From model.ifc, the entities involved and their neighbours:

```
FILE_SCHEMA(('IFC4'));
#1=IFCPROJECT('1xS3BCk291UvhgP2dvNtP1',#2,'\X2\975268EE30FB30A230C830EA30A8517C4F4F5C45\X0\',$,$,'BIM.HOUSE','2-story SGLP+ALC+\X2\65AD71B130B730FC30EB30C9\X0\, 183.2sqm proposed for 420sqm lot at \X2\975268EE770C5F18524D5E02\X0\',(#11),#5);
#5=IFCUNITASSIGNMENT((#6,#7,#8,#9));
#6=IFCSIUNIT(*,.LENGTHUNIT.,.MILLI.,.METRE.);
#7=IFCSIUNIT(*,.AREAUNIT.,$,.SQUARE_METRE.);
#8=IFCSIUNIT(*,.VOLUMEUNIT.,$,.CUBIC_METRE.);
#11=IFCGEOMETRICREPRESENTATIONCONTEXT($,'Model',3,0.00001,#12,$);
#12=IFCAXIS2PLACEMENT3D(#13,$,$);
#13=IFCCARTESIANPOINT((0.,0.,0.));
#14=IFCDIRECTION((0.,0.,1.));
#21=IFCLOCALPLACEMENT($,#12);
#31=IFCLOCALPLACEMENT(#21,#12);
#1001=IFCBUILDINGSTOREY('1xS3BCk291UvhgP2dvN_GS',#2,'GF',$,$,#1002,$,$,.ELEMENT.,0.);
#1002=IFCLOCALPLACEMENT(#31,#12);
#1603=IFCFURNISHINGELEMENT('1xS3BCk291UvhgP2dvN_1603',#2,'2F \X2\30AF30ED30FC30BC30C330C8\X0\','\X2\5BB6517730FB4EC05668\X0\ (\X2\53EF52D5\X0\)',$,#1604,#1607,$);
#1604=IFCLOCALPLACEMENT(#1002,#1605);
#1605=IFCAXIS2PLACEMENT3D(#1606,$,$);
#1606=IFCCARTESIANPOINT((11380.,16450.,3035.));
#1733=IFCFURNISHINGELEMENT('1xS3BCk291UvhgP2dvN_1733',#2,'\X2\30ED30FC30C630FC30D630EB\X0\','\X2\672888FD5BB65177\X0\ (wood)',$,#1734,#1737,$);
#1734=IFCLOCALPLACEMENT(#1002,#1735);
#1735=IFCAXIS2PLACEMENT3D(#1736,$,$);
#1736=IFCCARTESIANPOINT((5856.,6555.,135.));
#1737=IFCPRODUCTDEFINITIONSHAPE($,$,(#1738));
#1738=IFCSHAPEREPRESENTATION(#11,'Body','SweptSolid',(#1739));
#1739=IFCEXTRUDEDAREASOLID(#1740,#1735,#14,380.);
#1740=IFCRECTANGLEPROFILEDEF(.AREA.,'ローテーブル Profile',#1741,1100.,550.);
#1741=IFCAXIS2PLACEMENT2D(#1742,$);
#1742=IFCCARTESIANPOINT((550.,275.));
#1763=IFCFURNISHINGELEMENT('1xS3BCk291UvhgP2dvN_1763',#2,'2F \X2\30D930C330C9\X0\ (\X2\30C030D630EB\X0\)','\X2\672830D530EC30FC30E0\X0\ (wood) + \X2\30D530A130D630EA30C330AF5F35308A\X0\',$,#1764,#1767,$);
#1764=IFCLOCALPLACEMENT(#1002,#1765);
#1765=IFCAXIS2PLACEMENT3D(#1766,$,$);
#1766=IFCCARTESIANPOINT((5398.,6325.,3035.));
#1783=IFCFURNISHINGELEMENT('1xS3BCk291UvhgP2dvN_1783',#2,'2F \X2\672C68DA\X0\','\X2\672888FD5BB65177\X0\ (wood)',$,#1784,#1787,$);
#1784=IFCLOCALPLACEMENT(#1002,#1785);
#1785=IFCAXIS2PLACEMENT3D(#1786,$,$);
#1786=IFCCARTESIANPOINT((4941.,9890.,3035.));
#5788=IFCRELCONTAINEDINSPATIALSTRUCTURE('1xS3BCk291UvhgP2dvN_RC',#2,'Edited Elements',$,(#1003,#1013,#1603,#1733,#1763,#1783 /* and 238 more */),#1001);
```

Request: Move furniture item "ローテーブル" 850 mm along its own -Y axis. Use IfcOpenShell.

```python
import ifcopenshell
import ifcopenshell.api.geometry
import ifcopenshell.util.placement

model = ifcopenshell.open("model.ifc")

item = model.by_guid("1xS3BCk291UvhgP2dvN_1733")
matrix = ifcopenshell.util.placement.get_local_placement(item.ObjectPlacement)
matrix[:3, 3] -= matrix[:3, 1] * 850.0
ifcopenshell.api.geometry.edit_object_placement(model, product=item, matrix=matrix, is_si=False)

print(ifcopenshell.util.placement.get_local_placement(item.ObjectPlacement).round(3) + 0.0)

model.write("model_edited.ifc")
```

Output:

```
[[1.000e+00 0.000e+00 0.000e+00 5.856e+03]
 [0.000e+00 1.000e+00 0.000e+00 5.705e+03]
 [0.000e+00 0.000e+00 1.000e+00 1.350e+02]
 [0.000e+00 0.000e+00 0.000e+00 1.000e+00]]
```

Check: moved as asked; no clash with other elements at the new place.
